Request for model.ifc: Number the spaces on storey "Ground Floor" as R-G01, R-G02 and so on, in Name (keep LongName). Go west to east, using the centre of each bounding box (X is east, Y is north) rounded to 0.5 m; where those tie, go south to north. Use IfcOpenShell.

First a look at what the model holds.

```python
import ifcopenshell
import ifcopenshell.util.element
import ifcopenshell.util.placement

model = ifcopenshell.open("model.ifc")
print(model.schema)
storey = next(s for s in model.by_type("IfcBuildingStorey") if s.Name == "Ground Floor")
spaces = [e for e in ifcopenshell.util.element.get_decomposition(storey) if e.is_a("IfcSpace")]
for e in sorted(spaces, key=lambda e: e.id()):
    origin = ifcopenshell.util.placement.get_local_placement(e.ObjectPlacement)[:3, 3]
    print(e.id(), e.Name, e.LongName, origin.round(2) + 0.0, sep=" | ")
```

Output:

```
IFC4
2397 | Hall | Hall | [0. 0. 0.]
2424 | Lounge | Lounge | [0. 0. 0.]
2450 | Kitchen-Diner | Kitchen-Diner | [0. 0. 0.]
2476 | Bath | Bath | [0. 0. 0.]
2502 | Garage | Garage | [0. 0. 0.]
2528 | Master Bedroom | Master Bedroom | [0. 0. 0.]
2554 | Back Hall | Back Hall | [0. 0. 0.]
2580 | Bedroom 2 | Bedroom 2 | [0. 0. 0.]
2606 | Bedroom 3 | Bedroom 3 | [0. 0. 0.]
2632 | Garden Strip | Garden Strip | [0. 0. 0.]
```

```python
import ifcopenshell
import ifcopenshell.geom
import ifcopenshell.util.element
import ifcopenshell.util.shape

model = ifcopenshell.open("model.ifc")
settings = ifcopenshell.geom.settings()
settings.set("use-world-coords", True)


def centre(element):
    shape = ifcopenshell.geom.create_shape(settings, element)
    return ifcopenshell.util.shape.get_bbox_centroid(shape.geometry)


storey = next(s for s in model.by_type("IfcBuildingStorey") if s.Name == "Ground Floor")
spaces = [e for e in ifcopenshell.util.element.get_decomposition(storey) if e.is_a("IfcSpace")]

# Insertion points can sit at a corner or the storey origin, so sort by the geometry (in metres).
centres = {e: centre(e) for e in spaces}
spaces.sort(key=lambda e: (round(centres[e][0] / 0.5), centres[e][1]))

for i, e in enumerate(spaces, start=1):
    number = f"R-G{i:02d}"
    e.Name = number
    print(e.id(), number)

model.write("model_v2.ifc")
```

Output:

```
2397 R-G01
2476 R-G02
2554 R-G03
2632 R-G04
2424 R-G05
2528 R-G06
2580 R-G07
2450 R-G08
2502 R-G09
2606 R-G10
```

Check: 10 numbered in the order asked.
